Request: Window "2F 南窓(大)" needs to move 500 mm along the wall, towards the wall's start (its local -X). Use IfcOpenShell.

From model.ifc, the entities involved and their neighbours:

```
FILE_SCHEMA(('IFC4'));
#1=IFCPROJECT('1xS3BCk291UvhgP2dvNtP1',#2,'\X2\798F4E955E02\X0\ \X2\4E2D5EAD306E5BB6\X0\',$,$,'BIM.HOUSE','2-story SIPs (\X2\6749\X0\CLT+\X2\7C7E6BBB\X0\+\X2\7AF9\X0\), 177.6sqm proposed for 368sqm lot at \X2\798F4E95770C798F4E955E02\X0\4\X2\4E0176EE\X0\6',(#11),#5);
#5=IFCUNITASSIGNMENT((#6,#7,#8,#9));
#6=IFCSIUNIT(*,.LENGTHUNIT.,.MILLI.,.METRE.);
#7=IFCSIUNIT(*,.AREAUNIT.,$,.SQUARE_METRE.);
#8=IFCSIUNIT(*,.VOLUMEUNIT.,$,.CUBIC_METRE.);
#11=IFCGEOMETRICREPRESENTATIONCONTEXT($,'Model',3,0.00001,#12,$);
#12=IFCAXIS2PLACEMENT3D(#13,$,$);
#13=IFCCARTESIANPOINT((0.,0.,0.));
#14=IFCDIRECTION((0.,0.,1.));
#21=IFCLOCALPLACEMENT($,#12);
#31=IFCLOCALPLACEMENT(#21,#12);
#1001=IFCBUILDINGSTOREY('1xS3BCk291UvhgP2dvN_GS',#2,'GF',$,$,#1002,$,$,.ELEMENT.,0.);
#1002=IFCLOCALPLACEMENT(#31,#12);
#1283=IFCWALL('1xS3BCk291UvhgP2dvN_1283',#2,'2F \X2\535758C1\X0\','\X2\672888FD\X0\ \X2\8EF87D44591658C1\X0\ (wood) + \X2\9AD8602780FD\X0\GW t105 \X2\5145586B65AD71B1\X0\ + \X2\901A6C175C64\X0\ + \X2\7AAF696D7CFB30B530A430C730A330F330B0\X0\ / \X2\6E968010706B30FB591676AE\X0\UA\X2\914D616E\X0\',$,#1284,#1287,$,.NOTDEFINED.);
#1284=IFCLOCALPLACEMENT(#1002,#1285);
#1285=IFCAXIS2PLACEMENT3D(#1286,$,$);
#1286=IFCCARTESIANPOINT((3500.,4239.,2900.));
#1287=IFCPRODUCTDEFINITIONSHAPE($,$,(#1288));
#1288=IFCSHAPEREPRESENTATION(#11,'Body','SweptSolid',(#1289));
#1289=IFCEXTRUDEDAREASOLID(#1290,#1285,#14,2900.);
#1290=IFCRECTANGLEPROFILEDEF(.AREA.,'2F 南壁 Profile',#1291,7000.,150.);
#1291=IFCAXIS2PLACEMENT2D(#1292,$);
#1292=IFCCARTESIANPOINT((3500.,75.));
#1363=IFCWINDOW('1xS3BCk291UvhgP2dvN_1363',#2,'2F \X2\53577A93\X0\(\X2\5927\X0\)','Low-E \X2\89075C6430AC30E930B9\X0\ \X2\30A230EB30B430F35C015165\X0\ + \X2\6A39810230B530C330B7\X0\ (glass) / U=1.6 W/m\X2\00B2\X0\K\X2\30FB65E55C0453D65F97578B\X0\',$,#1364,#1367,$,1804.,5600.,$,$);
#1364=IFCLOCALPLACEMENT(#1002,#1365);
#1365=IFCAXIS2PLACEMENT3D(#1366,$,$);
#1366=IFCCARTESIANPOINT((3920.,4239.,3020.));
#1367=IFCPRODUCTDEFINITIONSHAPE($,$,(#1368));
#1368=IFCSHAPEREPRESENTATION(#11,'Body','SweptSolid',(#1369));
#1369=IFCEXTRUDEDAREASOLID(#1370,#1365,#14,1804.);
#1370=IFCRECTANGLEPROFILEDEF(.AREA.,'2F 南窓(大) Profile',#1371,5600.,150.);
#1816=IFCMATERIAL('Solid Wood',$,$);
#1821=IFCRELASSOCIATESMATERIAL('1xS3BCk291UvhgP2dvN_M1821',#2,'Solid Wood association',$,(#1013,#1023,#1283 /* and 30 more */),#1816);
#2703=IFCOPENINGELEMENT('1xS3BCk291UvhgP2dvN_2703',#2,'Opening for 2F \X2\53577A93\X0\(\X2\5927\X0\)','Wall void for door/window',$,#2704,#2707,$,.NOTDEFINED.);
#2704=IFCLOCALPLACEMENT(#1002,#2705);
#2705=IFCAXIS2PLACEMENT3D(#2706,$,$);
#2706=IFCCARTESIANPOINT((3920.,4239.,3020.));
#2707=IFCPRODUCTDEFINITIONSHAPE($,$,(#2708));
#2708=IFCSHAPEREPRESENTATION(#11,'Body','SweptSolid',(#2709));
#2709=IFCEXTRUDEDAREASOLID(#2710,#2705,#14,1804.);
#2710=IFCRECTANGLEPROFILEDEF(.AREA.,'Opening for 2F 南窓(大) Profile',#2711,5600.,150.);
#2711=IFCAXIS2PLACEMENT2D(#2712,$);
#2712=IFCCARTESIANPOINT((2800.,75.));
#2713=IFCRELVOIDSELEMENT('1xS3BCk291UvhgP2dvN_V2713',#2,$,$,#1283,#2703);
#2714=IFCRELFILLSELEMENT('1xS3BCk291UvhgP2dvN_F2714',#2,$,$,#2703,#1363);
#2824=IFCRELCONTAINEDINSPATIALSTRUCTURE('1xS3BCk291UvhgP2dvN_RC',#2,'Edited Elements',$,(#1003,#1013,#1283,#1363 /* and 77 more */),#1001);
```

```python
import ifcopenshell
import ifcopenshell.api.geometry
import ifcopenshell.util.placement
import ifcopenshell.util.unit

model = ifcopenshell.open("model.ifc")
unit_scale = ifcopenshell.util.unit.calculate_unit_scale(model)

window = model.by_guid("1xS3BCk291UvhgP2dvN_1363")
opening = window.FillsVoids[0].RelatingOpeningElement
wall = opening.VoidsElements[0].RelatingBuildingElement

wall_matrix = ifcopenshell.util.placement.get_local_placement(wall.ObjectPlacement)
shift = wall_matrix[:3, 0] * -0.5 / unit_scale
before = ifcopenshell.util.placement.get_local_placement(window.ObjectPlacement)[:3, 3].copy()

# The window is not placed relative to its opening, so move both.
for product in (opening, window):
    matrix = ifcopenshell.util.placement.get_local_placement(product.ObjectPlacement)
    matrix[:3, 3] += shift
    ifcopenshell.api.geometry.edit_object_placement(model, product=product, matrix=matrix, is_si=False)

after = ifcopenshell.util.placement.get_local_placement(window.ObjectPlacement)[:3, 3]
print("window moved by", (after - before).round(3) + 0.0)

model.write("model_edited.ifc")
```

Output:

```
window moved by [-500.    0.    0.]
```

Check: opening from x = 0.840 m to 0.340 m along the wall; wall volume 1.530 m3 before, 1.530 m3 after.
